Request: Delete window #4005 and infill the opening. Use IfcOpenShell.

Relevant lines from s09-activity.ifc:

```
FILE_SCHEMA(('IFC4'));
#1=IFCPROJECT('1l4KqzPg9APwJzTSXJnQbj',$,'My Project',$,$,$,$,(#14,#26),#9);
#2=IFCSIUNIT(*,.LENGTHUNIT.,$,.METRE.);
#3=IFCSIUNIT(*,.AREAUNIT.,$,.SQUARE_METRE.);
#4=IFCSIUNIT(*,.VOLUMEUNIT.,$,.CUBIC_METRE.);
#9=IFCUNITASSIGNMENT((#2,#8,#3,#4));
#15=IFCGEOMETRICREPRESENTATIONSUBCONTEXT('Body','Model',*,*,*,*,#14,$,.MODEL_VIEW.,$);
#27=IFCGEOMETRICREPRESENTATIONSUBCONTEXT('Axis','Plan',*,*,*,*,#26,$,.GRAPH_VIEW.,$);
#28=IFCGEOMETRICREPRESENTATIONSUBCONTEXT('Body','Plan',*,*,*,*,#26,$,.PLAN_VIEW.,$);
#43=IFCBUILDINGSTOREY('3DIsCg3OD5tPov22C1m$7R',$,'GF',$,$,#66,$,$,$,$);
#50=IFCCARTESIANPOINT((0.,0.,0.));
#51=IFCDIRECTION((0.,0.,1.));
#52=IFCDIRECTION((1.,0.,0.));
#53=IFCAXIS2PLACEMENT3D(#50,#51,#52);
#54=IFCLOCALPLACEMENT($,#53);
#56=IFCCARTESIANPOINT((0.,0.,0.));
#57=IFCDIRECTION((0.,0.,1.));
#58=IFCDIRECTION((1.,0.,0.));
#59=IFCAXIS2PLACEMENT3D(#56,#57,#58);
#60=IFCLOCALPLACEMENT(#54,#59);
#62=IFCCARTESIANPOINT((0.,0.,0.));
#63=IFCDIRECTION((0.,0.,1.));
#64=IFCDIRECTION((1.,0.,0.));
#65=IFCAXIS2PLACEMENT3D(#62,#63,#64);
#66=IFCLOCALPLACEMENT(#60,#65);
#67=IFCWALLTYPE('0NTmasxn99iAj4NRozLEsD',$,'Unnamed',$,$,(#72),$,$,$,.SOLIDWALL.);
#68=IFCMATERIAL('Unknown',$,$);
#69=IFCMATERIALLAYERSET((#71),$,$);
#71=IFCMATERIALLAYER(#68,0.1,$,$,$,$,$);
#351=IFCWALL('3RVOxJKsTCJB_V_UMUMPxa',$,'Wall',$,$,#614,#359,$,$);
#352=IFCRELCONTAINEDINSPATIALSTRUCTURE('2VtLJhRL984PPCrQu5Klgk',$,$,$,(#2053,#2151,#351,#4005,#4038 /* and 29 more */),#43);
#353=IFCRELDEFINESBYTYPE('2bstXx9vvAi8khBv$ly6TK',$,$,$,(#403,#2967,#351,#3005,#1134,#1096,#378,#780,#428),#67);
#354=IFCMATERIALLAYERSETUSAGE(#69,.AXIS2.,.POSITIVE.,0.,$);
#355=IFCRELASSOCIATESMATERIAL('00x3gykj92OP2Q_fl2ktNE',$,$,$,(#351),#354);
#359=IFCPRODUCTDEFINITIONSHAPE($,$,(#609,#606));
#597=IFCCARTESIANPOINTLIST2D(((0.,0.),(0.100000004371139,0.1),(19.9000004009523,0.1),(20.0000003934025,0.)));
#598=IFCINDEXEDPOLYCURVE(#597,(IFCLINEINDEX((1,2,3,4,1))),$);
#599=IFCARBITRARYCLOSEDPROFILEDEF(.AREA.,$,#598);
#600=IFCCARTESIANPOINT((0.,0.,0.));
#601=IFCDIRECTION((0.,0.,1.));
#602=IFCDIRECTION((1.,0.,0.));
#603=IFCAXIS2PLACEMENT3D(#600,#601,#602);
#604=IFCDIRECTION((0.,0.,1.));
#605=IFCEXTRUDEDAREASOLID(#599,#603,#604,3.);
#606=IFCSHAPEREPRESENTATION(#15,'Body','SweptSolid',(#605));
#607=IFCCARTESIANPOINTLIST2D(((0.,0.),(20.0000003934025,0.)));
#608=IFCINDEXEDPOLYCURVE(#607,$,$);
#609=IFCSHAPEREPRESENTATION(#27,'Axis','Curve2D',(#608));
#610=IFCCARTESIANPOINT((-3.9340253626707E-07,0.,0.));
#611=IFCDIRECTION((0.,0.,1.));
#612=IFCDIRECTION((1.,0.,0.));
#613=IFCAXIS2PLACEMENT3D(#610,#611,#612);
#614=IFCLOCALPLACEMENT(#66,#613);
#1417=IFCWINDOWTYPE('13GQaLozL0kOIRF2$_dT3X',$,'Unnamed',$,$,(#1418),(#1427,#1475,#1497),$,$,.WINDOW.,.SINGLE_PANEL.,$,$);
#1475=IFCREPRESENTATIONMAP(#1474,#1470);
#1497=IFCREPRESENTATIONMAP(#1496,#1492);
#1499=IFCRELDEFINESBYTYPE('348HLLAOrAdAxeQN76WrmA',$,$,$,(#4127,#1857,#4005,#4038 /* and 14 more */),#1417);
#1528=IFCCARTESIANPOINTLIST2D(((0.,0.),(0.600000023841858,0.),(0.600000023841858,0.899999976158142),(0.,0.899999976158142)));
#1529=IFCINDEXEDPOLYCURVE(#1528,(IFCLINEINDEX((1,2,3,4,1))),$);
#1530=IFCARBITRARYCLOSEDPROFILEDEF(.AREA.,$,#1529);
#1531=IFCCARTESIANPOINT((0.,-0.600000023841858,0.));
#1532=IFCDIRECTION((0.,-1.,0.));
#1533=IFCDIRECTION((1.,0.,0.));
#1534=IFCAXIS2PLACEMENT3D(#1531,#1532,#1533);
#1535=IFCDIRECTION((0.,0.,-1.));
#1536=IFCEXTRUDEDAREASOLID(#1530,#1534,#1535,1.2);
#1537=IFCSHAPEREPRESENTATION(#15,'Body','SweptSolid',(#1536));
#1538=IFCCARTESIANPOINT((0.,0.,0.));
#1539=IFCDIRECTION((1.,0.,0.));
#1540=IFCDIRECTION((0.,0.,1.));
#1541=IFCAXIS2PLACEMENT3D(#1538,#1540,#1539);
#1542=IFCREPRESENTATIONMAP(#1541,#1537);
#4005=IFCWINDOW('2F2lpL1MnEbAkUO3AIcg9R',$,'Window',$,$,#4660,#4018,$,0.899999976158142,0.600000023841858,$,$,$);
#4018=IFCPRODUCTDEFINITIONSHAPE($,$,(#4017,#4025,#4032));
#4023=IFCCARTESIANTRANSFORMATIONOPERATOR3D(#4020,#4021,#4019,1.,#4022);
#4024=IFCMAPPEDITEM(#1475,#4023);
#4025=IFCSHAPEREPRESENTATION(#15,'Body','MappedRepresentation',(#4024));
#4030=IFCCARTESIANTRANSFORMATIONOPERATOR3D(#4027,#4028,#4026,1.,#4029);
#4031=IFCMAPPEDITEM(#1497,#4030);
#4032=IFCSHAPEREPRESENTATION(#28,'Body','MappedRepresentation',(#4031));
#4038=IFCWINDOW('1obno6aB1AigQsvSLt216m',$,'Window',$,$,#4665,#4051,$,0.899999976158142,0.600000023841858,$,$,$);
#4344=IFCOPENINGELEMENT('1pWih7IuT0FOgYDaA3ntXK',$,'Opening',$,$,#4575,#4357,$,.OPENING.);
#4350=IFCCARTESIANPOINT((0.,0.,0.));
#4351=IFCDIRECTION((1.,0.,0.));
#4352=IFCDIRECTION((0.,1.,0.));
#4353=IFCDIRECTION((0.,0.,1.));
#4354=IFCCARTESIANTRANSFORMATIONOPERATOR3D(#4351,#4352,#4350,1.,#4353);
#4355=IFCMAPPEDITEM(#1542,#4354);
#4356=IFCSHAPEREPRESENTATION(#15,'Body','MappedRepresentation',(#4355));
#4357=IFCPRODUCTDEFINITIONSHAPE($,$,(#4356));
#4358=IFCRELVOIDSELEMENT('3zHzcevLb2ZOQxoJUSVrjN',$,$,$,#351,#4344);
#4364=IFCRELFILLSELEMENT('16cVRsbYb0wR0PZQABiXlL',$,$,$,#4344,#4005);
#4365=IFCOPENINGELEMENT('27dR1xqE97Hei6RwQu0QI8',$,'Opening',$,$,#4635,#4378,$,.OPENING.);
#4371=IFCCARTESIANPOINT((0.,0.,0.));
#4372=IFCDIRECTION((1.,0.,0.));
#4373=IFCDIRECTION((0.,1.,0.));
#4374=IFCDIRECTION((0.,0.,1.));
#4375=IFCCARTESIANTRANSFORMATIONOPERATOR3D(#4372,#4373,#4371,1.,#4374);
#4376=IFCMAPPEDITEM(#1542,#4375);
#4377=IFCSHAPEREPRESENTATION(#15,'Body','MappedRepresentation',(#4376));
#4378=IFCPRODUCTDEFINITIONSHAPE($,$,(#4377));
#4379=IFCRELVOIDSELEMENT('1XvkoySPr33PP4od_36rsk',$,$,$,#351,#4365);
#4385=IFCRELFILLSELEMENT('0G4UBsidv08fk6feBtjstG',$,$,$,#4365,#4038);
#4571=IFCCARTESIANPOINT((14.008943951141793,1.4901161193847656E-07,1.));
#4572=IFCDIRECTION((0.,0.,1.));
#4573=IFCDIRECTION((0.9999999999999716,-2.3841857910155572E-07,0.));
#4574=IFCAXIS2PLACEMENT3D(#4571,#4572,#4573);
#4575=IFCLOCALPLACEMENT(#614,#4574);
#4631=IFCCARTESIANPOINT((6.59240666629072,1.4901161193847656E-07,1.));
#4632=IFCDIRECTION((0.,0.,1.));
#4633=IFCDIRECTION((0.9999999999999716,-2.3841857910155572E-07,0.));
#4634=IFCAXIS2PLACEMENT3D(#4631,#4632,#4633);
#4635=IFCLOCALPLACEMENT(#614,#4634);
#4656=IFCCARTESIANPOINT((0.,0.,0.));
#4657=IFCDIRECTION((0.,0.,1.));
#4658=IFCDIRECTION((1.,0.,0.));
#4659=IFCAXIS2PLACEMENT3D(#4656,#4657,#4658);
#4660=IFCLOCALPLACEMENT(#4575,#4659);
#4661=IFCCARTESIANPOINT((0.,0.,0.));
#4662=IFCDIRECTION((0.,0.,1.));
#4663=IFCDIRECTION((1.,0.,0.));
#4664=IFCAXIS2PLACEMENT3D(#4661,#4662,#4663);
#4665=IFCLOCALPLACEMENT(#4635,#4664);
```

```python
import ifcopenshell
import ifcopenshell.api.feature
import ifcopenshell.api.root
import ifcopenshell.geom
import ifcopenshell.util.shape

model = ifcopenshell.open("s09-activity.ifc")
settings = ifcopenshell.geom.settings()


def volume(element):
    """Net volume in cubic metres, openings subtracted."""
    shape = ifcopenshell.geom.create_shape(settings, element)
    return ifcopenshell.util.shape.get_volume(shape.geometry)


window = model.by_guid("2F2lpL1MnEbAkUO3AIcg9R")
opening = window.FillsVoids[0].RelatingOpeningElement
wall = opening.VoidsElements[0].RelatingBuildingElement
before = volume(wall)

ifcopenshell.api.root.remove_product(model, product=window)
ifcopenshell.api.feature.remove_feature(model, feature=opening)

after = volume(wall)

print(f"wall volume {before:.3f} -> {after:.3f} m3")

model.write("s09-activity_updated.ifc")
```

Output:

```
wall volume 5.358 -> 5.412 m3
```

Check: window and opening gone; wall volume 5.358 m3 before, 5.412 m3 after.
